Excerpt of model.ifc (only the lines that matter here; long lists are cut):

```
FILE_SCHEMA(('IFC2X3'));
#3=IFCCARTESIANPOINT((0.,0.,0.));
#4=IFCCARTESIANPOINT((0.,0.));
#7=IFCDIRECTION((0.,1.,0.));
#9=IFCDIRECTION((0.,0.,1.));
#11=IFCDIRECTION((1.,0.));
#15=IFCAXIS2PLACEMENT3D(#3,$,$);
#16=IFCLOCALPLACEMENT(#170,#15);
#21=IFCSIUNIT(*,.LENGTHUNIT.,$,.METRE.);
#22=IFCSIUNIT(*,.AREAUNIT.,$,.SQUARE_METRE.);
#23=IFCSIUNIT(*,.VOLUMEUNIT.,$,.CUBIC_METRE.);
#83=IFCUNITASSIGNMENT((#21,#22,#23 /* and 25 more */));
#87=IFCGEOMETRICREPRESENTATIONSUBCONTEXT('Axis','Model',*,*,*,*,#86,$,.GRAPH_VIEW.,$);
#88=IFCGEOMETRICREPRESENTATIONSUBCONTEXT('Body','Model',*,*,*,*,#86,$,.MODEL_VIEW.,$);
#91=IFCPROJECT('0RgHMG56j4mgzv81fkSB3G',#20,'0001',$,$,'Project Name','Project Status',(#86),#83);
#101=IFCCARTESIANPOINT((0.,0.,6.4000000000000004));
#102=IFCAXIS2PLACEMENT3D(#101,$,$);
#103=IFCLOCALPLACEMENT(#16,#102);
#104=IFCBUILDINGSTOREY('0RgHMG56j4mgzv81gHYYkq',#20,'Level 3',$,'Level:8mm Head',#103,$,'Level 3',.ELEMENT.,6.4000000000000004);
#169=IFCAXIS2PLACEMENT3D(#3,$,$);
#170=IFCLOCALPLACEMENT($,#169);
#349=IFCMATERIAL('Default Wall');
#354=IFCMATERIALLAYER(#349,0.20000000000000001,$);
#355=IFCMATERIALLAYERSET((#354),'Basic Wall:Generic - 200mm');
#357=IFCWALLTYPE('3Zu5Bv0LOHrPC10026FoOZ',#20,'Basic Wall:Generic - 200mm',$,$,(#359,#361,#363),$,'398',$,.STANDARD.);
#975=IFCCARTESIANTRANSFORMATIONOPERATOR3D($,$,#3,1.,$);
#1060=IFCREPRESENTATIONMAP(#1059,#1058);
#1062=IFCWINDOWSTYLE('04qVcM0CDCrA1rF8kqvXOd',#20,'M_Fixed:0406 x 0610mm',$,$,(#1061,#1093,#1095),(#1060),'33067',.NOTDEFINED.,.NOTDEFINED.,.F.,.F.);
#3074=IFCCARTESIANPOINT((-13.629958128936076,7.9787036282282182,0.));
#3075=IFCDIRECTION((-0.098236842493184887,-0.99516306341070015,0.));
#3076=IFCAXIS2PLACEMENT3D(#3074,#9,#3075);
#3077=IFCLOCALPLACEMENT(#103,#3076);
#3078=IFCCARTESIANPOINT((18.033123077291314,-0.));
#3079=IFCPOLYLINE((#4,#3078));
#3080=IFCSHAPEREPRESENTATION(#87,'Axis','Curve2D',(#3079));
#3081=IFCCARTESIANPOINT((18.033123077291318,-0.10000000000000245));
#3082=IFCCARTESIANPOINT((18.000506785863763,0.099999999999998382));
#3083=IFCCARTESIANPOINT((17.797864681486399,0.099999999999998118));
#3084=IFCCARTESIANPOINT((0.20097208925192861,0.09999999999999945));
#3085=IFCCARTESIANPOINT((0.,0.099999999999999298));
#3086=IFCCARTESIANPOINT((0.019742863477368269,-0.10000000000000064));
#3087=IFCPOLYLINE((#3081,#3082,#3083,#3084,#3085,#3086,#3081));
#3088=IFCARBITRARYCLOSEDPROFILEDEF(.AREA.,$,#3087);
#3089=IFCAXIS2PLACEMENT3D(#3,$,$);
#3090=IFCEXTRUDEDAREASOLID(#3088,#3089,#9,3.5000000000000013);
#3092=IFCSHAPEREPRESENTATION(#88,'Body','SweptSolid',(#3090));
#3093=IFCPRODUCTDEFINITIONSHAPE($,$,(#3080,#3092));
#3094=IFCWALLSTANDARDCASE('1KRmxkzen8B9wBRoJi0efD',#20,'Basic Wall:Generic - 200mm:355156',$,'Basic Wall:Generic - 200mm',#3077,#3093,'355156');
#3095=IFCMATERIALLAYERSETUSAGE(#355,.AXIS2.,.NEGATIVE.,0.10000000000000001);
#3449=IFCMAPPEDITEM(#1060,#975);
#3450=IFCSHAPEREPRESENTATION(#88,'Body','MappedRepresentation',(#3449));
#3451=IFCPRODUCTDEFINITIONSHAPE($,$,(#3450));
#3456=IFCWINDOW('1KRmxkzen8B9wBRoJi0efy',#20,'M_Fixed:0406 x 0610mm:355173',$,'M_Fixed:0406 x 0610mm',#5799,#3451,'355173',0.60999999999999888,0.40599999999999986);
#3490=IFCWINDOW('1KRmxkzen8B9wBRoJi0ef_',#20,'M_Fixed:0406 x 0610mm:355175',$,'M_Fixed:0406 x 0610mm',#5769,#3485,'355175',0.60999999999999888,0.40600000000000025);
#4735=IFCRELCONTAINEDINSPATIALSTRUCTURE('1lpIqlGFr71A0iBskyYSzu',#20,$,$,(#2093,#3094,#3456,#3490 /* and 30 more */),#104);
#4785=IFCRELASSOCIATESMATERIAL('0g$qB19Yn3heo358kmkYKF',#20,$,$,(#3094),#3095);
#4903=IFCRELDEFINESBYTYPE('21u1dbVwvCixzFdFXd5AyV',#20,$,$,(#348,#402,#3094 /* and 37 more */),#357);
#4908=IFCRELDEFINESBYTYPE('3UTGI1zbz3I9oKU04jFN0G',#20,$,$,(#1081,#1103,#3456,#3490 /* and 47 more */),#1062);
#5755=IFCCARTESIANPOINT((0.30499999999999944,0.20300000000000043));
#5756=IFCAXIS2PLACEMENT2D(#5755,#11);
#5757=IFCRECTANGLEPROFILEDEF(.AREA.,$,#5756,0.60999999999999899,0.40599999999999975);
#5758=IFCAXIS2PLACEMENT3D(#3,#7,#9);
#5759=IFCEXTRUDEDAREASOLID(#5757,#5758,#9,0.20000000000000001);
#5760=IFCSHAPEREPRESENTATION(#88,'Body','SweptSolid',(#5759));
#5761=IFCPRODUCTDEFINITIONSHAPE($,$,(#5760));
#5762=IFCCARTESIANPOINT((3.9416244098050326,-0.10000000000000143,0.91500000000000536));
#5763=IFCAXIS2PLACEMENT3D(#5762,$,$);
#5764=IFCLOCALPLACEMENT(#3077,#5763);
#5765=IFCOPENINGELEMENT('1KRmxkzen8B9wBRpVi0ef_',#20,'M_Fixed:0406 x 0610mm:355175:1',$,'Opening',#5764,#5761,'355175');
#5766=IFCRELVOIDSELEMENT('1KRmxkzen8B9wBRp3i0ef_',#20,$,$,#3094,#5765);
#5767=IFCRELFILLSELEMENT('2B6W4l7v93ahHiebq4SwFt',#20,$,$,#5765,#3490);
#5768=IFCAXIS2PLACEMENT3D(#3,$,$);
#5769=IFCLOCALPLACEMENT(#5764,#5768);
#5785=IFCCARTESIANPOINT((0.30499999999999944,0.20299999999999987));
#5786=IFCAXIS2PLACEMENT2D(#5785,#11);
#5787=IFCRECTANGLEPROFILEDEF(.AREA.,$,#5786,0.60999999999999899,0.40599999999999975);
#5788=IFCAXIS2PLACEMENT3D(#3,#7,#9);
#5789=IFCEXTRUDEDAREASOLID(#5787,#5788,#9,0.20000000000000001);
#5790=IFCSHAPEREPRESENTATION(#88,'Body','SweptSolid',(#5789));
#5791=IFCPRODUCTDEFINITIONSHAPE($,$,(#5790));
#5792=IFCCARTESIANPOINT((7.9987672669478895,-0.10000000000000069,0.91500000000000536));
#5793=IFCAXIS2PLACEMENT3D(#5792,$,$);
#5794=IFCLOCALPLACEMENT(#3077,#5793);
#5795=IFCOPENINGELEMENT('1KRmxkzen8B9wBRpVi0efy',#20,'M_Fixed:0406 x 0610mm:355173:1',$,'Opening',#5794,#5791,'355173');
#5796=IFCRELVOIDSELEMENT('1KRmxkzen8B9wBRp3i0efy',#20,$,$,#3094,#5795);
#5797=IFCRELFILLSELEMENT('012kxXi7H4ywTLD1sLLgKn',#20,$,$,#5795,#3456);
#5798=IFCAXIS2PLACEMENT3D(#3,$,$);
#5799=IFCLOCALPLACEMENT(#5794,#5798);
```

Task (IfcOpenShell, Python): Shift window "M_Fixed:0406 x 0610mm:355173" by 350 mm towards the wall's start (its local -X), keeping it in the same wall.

```python
import ifcopenshell
import ifcopenshell.api.geometry
import ifcopenshell.util.placement
import ifcopenshell.util.unit

model = ifcopenshell.open("model.ifc")
unit_scale = ifcopenshell.util.unit.calculate_unit_scale(model)

window = model.by_id(3456)
opening = window.FillsVoids[0].RelatingOpeningElement
wall = opening.VoidsElements[0].RelatingBuildingElement

wall_matrix = ifcopenshell.util.placement.get_local_placement(wall.ObjectPlacement)
shift = wall_matrix[:3, 0] * -0.35 / unit_scale
before = ifcopenshell.util.placement.get_local_placement(window.ObjectPlacement)[:3, 3].copy()

# The window is placed relative to its opening, so it follows when the opening moves.
matrix = ifcopenshell.util.placement.get_local_placement(opening.ObjectPlacement)
matrix[:3, 3] += shift
ifcopenshell.api.geometry.edit_object_placement(
    model, product=opening, matrix=matrix, is_si=False, should_transform_children=True
)

after = ifcopenshell.util.placement.get_local_placement(window.ObjectPlacement)[:3, 3]
print("window moved by", (after - before).round(3) + 0.0)

model.write("model-out.ifc")
```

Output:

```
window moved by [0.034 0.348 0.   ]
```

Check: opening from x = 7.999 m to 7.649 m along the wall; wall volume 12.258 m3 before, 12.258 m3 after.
